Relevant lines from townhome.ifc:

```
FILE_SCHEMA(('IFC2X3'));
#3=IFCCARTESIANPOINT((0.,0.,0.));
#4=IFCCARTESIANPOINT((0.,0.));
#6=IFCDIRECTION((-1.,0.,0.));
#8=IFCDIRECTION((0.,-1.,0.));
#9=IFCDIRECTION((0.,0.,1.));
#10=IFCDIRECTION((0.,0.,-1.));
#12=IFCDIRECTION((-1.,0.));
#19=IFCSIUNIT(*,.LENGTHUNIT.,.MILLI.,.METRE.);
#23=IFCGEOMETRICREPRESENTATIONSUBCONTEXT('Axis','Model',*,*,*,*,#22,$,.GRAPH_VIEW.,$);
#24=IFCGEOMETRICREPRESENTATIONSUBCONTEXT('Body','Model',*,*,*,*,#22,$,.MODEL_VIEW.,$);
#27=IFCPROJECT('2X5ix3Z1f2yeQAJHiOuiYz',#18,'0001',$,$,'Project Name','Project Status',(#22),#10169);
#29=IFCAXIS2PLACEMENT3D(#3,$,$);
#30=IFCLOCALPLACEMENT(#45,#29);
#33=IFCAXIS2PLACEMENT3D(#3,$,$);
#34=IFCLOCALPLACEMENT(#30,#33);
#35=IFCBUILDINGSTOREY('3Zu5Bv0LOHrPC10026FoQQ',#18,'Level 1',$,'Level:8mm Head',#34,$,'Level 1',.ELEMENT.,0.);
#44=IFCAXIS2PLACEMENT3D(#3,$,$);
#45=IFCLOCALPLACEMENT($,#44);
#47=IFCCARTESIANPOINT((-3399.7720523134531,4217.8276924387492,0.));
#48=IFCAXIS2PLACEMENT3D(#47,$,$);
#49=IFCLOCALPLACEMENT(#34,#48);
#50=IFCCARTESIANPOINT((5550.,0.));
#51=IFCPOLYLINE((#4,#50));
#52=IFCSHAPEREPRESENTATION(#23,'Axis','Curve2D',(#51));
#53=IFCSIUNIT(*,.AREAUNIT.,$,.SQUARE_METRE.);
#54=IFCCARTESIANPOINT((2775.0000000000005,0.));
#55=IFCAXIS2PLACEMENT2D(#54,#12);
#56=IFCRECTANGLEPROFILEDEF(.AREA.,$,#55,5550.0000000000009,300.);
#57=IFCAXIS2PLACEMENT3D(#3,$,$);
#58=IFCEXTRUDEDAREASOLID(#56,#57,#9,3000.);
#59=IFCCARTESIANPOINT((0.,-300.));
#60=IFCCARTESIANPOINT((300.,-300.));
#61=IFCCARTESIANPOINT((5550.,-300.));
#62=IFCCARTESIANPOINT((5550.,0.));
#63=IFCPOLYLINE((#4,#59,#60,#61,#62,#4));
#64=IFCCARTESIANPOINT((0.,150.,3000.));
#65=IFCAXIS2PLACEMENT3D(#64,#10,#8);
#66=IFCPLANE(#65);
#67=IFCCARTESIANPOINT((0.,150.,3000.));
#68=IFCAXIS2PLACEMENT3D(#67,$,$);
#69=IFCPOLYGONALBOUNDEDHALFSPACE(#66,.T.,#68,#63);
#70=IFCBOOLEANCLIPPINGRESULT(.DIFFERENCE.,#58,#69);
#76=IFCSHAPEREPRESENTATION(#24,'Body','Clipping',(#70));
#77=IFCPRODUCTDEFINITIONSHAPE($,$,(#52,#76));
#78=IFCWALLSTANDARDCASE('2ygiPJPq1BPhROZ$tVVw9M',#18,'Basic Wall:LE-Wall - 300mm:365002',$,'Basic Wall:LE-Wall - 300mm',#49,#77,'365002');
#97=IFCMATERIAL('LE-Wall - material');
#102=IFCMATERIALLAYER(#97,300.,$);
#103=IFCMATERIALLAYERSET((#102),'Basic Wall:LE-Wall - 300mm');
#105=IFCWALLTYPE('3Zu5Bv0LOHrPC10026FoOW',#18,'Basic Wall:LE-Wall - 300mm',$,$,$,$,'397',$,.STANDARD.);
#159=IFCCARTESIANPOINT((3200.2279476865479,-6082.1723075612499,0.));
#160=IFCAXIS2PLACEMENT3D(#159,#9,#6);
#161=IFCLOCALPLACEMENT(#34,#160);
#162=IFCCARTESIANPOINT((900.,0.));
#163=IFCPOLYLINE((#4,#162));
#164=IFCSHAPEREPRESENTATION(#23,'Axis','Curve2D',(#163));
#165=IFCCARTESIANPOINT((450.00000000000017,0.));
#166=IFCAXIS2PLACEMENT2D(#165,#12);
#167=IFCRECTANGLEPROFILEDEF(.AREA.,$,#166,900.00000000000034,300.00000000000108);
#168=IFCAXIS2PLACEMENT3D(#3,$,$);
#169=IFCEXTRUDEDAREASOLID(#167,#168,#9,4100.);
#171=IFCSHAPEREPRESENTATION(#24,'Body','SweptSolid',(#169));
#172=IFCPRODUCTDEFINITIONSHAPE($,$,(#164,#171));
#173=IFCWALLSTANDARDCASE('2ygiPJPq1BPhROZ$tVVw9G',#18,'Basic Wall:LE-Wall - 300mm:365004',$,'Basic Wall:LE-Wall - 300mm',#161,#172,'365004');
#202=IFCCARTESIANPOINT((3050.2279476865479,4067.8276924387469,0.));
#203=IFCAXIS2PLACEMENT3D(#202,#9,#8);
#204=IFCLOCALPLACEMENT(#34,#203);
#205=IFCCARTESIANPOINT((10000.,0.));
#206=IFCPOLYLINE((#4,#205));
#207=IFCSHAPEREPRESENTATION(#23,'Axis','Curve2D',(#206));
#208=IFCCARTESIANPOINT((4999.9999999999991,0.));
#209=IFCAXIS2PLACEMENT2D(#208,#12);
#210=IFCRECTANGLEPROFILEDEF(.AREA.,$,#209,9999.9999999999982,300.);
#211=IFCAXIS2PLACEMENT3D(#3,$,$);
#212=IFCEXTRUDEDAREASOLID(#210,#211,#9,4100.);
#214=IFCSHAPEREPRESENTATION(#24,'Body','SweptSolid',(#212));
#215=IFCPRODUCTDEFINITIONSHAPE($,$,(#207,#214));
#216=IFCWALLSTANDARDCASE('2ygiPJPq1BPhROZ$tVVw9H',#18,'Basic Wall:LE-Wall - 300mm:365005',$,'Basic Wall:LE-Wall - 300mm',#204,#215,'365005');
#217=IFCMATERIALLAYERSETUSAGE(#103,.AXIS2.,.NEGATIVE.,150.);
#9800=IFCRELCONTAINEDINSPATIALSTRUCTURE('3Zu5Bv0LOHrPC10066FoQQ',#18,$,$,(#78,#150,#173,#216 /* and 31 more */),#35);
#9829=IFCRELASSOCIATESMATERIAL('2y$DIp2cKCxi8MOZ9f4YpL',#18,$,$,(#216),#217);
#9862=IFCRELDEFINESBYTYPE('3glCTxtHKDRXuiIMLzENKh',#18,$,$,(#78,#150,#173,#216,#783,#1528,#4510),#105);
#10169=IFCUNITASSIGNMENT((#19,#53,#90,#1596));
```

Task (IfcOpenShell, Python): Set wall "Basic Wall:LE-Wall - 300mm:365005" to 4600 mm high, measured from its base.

```python
import ifcopenshell
import ifcopenshell.geom
import ifcopenshell.util.representation
import ifcopenshell.util.shape
import ifcopenshell.util.unit

model = ifcopenshell.open("townhome.ifc")
unit_scale = ifcopenshell.util.unit.calculate_unit_scale(model)
settings = ifcopenshell.geom.settings()


def volume(element):
    """Net volume in cubic metres, openings subtracted."""
    shape = ifcopenshell.geom.create_shape(settings, element)
    return ifcopenshell.util.shape.get_volume(shape.geometry)


wall = model.by_id(216)
before = volume(wall)

body = ifcopenshell.util.representation.get_representation(wall, "Model", "Body")
solid = body.Items[0]
old_height = solid.Depth
solid.Depth = 4.6 / unit_scale
after = volume(wall)

print(f"height {old_height:g} -> {solid.Depth:g}, volume {before:.3f} -> {after:.3f} m3")

model.write("townhome_rev.ifc")
```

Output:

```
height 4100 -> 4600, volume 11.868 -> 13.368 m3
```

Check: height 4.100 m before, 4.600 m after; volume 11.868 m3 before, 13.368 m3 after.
